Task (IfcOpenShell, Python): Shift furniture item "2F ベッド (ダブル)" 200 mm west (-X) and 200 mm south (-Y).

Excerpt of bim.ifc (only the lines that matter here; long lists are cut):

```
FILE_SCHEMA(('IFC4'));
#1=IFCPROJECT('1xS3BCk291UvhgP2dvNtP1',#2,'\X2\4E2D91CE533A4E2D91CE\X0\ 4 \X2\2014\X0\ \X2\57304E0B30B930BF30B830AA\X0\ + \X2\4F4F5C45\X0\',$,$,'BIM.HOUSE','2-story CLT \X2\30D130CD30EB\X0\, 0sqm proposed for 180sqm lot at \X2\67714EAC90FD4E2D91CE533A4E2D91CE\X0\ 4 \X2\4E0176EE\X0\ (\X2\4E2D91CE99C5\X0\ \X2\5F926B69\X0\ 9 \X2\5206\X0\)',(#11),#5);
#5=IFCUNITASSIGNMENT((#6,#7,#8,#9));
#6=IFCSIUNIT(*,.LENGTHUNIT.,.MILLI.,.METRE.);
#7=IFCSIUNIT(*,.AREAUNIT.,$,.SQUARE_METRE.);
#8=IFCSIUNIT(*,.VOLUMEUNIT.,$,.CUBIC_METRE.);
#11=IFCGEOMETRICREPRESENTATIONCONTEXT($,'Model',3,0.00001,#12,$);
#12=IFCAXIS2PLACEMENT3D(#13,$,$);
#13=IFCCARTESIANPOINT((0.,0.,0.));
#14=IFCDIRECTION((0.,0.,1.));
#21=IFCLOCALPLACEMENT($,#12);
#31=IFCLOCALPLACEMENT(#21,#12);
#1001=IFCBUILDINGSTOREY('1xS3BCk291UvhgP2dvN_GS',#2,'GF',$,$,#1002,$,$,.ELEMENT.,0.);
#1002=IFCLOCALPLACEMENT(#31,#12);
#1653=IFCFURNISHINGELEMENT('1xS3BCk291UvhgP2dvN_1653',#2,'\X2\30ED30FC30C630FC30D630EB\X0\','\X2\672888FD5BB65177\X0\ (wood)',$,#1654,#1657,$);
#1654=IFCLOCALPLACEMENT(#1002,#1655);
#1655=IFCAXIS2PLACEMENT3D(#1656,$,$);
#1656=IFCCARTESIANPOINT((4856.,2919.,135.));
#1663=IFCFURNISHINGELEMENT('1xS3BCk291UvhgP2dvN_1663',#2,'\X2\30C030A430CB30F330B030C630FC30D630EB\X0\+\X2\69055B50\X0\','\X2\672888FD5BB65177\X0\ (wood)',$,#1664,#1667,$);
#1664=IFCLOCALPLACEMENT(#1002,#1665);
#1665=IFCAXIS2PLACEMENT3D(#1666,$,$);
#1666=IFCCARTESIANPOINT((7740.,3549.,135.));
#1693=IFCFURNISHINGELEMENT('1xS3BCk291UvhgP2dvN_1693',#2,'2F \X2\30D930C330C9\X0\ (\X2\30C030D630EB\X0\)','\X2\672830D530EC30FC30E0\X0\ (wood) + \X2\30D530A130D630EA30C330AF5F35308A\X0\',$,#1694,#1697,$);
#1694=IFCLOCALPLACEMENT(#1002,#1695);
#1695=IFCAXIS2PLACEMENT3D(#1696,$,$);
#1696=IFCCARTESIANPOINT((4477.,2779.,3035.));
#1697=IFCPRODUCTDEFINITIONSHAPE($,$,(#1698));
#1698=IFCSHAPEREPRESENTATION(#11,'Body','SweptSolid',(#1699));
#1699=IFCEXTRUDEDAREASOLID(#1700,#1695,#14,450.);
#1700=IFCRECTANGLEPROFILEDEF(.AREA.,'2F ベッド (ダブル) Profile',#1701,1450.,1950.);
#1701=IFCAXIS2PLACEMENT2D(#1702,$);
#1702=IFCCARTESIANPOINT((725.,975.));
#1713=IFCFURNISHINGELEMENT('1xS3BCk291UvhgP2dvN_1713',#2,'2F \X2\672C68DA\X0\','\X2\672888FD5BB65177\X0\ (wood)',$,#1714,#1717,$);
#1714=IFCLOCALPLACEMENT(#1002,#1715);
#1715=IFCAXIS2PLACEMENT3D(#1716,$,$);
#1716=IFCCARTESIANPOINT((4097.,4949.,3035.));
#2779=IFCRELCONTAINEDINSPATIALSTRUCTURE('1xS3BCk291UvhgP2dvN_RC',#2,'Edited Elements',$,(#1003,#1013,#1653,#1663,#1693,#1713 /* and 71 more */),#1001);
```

```python
import ifcopenshell
import ifcopenshell.api.geometry
import ifcopenshell.util.placement

model = ifcopenshell.open("bim.ifc")

item = model.by_guid("1xS3BCk291UvhgP2dvN_1693")
matrix = ifcopenshell.util.placement.get_local_placement(item.ObjectPlacement)
matrix[0, 3] -= 200.0
matrix[1, 3] -= 200.0
ifcopenshell.api.geometry.edit_object_placement(model, product=item, matrix=matrix, is_si=False)

print(ifcopenshell.util.placement.get_local_placement(item.ObjectPlacement).round(3) + 0.0)

model.write("bim-out.ifc")
```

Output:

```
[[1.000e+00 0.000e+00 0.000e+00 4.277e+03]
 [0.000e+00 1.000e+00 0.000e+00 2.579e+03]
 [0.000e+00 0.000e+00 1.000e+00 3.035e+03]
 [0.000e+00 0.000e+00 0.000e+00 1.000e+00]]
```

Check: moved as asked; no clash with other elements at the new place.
